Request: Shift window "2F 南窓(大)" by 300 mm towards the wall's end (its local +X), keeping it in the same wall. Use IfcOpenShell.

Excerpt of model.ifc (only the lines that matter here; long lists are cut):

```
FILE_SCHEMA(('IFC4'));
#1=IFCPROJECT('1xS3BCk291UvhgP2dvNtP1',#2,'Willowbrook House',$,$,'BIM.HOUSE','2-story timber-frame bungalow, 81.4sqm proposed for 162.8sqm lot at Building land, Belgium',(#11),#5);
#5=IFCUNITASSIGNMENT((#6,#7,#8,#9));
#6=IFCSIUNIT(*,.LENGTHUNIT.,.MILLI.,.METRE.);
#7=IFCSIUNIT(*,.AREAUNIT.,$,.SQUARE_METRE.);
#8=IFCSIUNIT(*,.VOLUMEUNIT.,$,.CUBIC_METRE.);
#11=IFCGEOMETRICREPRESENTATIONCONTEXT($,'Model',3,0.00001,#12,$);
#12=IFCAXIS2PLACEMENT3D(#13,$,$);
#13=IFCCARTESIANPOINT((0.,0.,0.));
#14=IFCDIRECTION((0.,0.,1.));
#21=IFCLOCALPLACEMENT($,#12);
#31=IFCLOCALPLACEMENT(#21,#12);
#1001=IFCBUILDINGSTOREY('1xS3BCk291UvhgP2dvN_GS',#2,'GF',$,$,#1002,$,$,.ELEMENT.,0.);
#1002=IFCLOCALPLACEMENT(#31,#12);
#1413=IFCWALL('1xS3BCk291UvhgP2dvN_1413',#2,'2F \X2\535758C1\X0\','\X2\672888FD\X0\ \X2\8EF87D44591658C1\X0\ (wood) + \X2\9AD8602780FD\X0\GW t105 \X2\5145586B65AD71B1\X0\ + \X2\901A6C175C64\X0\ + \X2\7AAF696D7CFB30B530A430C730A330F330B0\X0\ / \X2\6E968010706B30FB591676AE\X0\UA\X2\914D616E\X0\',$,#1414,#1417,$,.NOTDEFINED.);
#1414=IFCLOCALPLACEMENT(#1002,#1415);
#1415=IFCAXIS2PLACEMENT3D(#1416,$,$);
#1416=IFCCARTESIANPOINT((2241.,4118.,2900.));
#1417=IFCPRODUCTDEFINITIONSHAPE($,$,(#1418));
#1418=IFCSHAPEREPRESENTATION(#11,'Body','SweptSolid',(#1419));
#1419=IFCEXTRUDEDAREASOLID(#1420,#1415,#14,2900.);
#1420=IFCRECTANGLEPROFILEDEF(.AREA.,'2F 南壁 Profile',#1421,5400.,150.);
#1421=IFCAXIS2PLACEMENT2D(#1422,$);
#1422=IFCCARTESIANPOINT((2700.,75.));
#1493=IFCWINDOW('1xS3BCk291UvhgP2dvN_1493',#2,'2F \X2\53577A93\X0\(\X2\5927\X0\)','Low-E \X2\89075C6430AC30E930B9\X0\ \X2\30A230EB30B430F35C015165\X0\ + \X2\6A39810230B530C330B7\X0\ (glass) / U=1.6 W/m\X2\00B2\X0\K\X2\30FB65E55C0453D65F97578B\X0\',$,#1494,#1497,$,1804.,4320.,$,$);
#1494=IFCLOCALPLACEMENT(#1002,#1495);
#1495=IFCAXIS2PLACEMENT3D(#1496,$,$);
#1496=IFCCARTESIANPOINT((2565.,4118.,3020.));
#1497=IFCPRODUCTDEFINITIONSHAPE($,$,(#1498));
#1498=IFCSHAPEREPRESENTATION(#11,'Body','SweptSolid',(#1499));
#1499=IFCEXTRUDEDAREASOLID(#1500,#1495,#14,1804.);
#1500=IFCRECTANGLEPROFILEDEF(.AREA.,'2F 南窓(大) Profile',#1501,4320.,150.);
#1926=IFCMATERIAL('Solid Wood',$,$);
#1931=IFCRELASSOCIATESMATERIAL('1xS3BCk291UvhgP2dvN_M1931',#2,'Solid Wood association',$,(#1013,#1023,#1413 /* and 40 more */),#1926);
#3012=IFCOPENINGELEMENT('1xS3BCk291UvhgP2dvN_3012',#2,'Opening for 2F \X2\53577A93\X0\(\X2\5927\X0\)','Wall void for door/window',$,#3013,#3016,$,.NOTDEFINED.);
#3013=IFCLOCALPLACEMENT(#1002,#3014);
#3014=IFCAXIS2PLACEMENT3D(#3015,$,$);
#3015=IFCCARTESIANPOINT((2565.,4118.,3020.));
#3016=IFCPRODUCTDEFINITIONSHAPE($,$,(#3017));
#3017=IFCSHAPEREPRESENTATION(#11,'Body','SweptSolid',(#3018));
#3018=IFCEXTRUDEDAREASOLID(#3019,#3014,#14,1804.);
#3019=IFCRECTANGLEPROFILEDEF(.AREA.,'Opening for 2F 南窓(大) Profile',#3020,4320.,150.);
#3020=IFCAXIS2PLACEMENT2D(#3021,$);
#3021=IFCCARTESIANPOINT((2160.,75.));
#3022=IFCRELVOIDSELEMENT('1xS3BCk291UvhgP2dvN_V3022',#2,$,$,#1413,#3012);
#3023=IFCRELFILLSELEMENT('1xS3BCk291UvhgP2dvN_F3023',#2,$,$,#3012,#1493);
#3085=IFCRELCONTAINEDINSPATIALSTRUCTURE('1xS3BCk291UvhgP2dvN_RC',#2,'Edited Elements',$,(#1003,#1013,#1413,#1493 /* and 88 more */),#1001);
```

```python
import ifcopenshell
import ifcopenshell.api.geometry
import ifcopenshell.util.placement
import ifcopenshell.util.unit

model = ifcopenshell.open("model.ifc")
unit_scale = ifcopenshell.util.unit.calculate_unit_scale(model)

window = model.by_id(1493)
opening = window.FillsVoids[0].RelatingOpeningElement
wall = opening.VoidsElements[0].RelatingBuildingElement

wall_matrix = ifcopenshell.util.placement.get_local_placement(wall.ObjectPlacement)
shift = wall_matrix[:3, 0] * 0.3 / unit_scale
before = ifcopenshell.util.placement.get_local_placement(window.ObjectPlacement)[:3, 3].copy()

# The window is not placed relative to its opening, so move both.
for product in (opening, window):
    matrix = ifcopenshell.util.placement.get_local_placement(product.ObjectPlacement)
    matrix[:3, 3] += shift
    ifcopenshell.api.geometry.edit_object_placement(model, product=product, matrix=matrix, is_si=False)

after = ifcopenshell.util.placement.get_local_placement(window.ObjectPlacement)[:3, 3]
print("window moved by", (after - before).round(3) + 0.0)

model.write("model-out.ifc")
```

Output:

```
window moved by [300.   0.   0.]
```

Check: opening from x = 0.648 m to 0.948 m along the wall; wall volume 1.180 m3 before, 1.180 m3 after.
